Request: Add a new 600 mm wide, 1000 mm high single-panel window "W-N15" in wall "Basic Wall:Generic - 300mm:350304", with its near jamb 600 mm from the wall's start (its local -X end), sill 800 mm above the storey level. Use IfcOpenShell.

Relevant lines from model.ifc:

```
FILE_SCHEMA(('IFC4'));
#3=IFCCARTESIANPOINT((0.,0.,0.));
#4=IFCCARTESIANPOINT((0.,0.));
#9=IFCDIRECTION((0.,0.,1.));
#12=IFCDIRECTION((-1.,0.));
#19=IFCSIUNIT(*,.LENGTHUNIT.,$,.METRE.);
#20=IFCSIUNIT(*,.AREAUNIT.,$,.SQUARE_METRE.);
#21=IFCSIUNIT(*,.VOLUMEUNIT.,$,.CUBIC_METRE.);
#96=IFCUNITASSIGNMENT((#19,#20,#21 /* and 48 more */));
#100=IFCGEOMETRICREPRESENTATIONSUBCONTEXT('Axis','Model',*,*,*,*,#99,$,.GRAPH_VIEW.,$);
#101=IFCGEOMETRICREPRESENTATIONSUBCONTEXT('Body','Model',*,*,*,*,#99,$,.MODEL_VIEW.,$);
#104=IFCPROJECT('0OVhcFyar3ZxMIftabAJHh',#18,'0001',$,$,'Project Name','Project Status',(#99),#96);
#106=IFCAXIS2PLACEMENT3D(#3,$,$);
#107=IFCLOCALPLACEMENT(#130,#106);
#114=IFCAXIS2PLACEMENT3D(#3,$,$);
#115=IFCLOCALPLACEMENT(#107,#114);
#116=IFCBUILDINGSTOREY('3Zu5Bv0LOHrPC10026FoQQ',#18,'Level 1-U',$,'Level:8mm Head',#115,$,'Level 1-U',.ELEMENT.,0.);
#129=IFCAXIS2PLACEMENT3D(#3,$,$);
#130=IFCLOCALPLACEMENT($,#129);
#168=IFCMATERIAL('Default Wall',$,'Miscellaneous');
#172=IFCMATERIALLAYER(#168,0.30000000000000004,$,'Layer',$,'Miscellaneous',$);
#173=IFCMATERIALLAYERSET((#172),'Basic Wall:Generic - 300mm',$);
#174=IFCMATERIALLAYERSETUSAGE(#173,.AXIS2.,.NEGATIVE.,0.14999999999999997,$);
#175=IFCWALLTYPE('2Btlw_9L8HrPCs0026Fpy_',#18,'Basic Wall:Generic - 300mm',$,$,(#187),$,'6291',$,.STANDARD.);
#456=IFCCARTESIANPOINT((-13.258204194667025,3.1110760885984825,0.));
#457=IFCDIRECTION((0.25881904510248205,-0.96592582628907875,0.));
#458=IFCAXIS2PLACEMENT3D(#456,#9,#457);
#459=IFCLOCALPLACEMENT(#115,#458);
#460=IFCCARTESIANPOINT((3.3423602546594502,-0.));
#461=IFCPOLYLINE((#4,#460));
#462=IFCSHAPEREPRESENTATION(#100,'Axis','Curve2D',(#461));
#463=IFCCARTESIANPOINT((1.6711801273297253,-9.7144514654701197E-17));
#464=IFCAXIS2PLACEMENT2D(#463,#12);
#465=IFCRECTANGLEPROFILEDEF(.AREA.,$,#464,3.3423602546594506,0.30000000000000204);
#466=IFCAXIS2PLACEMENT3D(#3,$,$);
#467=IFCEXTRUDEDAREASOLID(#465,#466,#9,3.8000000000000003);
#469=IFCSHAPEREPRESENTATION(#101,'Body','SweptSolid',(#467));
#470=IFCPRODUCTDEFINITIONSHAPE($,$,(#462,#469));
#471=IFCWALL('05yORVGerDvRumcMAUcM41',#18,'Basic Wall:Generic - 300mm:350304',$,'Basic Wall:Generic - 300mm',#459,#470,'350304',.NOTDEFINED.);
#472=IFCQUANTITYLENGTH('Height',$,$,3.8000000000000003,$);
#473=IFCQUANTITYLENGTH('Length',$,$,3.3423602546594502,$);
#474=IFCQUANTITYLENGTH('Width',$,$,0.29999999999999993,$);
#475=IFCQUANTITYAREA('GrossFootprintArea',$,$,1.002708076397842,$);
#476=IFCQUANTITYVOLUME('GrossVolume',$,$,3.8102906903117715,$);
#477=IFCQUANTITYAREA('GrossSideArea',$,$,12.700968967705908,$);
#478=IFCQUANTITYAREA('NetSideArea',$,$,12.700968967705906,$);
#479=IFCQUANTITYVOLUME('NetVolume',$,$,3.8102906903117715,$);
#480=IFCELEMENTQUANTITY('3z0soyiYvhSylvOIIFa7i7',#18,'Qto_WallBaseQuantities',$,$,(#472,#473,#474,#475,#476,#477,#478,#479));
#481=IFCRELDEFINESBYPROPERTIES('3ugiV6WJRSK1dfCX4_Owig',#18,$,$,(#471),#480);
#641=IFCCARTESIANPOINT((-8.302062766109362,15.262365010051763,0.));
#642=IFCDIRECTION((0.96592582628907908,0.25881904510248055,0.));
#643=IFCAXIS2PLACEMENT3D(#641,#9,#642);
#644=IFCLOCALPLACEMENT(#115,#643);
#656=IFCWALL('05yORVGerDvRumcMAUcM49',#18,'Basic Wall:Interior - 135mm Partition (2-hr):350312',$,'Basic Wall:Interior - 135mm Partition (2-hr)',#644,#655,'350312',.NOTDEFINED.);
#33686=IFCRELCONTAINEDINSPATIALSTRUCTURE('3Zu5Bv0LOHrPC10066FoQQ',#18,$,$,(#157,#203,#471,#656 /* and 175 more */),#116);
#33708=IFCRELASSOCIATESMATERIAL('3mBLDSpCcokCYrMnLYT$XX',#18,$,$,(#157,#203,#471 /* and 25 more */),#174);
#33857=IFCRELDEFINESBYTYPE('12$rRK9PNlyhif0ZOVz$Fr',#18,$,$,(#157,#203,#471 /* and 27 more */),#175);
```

```python
import numpy as np
import ifcopenshell
import ifcopenshell.api.feature
import ifcopenshell.api.geometry
import ifcopenshell.api.pset
import ifcopenshell.api.root
import ifcopenshell.api.spatial
import ifcopenshell.geom
import ifcopenshell.util.element
import ifcopenshell.util.placement
import ifcopenshell.util.representation
import ifcopenshell.util.shape
import ifcopenshell.util.unit

model = ifcopenshell.open("model.ifc")
unit_scale = ifcopenshell.util.unit.calculate_unit_scale(model)
area_scale = ifcopenshell.util.unit.calculate_unit_scale(model, "AREAUNIT")
volume_scale = ifcopenshell.util.unit.calculate_unit_scale(model, "VOLUMEUNIT")
settings = ifcopenshell.geom.settings()


def volume(element):
    """Net volume in cubic metres, openings subtracted."""
    shape = ifcopenshell.geom.create_shape(settings, element)
    return ifcopenshell.util.shape.get_volume(shape.geometry)


wall = model.by_id(471)
storey = ifcopenshell.util.element.get_container(wall, ifc_class="IfcBuildingStorey")
context = ifcopenshell.util.representation.get_context(model, "Model", "Body", "MODEL_VIEW")
before = volume(wall)

width, height, from_end, sill = 0.6, 1, 0.6, 0.8  # metres

# The wall runs along its own X axis, and the end named is its -X end.
wall_shape = ifcopenshell.geom.create_shape(settings, wall)
x, y, z = ifcopenshell.util.shape.get_vertices(wall_shape.geometry).T
start = x.min() + from_end
face, thickness = float(y.min()), float(y.max() - y.min())
wall_matrix = ifcopenshell.util.placement.get_local_placement(wall.ObjectPlacement)
level = ifcopenshell.util.placement.get_local_placement(storey.ObjectPlacement)[2, 3]


def in_wall(x, y):
    """Placement at x, y metres in the wall's axes, at sill height."""
    matrix = wall_matrix.copy()
    matrix[:, 3] = wall_matrix @ np.array([x / unit_scale, y / unit_scale, 0.0, 1.0])
    matrix[2, 3] = level + sill / unit_scale
    return matrix


# Opening: a box that overshoots both wall faces by 50 mm.
opening = ifcopenshell.api.root.create_entity(model, ifc_class="IfcOpeningElement", predefined_type="OPENING")
box = ifcopenshell.api.geometry.add_wall_representation(
    model, context=context, length=width, height=height, thickness=thickness + 0.1
)
ifcopenshell.api.geometry.assign_representation(model, product=opening, representation=box)
ifcopenshell.api.geometry.edit_object_placement(model, product=opening, matrix=in_wall(start, face - 0.05), is_si=False)
ifcopenshell.api.feature.add_feature(model, feature=opening, element=wall)

window = ifcopenshell.api.root.create_entity(model, ifc_class="IfcWindow", name="W-N15", predefined_type="WINDOW")
window.OverallWidth, window.OverallHeight = width / unit_scale, height / unit_scale
window.PartitioningType = "SINGLE_PANEL"
body = ifcopenshell.api.geometry.add_window_representation(
    model,
    context=context,
    overall_width=window.OverallWidth,
    overall_height=window.OverallHeight,
    partition_type="SINGLE_PANEL",
)
ifcopenshell.api.geometry.assign_representation(model, product=window, representation=body)
ifcopenshell.api.spatial.assign_container(model, products=[window], relating_structure=storey)
ifcopenshell.api.feature.add_filling(model, opening=opening, element=window)

# Centre the window in the wall's thickness.
ifcopenshell.api.geometry.edit_object_placement(model, product=window, matrix=in_wall(start, face), is_si=False)
window_shape = ifcopenshell.geom.create_shape(settings, window)
depth = ifcopenshell.util.shape.get_vertices(window_shape.geometry)[:, 1]
offset = face + thickness / 2 - (depth.min() + depth.max()) / 2
ifcopenshell.api.geometry.edit_object_placement(model, product=window, matrix=in_wall(start, offset), is_si=False)

after = volume(wall)

# Update the wall's stored quantities.
qto = model.by_id(ifcopenshell.util.element.get_pset(wall, "Qto_WallBaseQuantities", should_inherit=False)["id"])
ifcopenshell.api.pset.edit_qto(model, qto=qto, properties={
    "NetSideArea": after / thickness / area_scale,
    "NetVolume": after / volume_scale,
})

print(f"wall volume {before:.3f} -> {after:.3f} m3")

model.write("model_edited.ifc")
```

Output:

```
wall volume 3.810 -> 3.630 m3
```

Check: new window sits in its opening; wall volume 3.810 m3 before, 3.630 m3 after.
